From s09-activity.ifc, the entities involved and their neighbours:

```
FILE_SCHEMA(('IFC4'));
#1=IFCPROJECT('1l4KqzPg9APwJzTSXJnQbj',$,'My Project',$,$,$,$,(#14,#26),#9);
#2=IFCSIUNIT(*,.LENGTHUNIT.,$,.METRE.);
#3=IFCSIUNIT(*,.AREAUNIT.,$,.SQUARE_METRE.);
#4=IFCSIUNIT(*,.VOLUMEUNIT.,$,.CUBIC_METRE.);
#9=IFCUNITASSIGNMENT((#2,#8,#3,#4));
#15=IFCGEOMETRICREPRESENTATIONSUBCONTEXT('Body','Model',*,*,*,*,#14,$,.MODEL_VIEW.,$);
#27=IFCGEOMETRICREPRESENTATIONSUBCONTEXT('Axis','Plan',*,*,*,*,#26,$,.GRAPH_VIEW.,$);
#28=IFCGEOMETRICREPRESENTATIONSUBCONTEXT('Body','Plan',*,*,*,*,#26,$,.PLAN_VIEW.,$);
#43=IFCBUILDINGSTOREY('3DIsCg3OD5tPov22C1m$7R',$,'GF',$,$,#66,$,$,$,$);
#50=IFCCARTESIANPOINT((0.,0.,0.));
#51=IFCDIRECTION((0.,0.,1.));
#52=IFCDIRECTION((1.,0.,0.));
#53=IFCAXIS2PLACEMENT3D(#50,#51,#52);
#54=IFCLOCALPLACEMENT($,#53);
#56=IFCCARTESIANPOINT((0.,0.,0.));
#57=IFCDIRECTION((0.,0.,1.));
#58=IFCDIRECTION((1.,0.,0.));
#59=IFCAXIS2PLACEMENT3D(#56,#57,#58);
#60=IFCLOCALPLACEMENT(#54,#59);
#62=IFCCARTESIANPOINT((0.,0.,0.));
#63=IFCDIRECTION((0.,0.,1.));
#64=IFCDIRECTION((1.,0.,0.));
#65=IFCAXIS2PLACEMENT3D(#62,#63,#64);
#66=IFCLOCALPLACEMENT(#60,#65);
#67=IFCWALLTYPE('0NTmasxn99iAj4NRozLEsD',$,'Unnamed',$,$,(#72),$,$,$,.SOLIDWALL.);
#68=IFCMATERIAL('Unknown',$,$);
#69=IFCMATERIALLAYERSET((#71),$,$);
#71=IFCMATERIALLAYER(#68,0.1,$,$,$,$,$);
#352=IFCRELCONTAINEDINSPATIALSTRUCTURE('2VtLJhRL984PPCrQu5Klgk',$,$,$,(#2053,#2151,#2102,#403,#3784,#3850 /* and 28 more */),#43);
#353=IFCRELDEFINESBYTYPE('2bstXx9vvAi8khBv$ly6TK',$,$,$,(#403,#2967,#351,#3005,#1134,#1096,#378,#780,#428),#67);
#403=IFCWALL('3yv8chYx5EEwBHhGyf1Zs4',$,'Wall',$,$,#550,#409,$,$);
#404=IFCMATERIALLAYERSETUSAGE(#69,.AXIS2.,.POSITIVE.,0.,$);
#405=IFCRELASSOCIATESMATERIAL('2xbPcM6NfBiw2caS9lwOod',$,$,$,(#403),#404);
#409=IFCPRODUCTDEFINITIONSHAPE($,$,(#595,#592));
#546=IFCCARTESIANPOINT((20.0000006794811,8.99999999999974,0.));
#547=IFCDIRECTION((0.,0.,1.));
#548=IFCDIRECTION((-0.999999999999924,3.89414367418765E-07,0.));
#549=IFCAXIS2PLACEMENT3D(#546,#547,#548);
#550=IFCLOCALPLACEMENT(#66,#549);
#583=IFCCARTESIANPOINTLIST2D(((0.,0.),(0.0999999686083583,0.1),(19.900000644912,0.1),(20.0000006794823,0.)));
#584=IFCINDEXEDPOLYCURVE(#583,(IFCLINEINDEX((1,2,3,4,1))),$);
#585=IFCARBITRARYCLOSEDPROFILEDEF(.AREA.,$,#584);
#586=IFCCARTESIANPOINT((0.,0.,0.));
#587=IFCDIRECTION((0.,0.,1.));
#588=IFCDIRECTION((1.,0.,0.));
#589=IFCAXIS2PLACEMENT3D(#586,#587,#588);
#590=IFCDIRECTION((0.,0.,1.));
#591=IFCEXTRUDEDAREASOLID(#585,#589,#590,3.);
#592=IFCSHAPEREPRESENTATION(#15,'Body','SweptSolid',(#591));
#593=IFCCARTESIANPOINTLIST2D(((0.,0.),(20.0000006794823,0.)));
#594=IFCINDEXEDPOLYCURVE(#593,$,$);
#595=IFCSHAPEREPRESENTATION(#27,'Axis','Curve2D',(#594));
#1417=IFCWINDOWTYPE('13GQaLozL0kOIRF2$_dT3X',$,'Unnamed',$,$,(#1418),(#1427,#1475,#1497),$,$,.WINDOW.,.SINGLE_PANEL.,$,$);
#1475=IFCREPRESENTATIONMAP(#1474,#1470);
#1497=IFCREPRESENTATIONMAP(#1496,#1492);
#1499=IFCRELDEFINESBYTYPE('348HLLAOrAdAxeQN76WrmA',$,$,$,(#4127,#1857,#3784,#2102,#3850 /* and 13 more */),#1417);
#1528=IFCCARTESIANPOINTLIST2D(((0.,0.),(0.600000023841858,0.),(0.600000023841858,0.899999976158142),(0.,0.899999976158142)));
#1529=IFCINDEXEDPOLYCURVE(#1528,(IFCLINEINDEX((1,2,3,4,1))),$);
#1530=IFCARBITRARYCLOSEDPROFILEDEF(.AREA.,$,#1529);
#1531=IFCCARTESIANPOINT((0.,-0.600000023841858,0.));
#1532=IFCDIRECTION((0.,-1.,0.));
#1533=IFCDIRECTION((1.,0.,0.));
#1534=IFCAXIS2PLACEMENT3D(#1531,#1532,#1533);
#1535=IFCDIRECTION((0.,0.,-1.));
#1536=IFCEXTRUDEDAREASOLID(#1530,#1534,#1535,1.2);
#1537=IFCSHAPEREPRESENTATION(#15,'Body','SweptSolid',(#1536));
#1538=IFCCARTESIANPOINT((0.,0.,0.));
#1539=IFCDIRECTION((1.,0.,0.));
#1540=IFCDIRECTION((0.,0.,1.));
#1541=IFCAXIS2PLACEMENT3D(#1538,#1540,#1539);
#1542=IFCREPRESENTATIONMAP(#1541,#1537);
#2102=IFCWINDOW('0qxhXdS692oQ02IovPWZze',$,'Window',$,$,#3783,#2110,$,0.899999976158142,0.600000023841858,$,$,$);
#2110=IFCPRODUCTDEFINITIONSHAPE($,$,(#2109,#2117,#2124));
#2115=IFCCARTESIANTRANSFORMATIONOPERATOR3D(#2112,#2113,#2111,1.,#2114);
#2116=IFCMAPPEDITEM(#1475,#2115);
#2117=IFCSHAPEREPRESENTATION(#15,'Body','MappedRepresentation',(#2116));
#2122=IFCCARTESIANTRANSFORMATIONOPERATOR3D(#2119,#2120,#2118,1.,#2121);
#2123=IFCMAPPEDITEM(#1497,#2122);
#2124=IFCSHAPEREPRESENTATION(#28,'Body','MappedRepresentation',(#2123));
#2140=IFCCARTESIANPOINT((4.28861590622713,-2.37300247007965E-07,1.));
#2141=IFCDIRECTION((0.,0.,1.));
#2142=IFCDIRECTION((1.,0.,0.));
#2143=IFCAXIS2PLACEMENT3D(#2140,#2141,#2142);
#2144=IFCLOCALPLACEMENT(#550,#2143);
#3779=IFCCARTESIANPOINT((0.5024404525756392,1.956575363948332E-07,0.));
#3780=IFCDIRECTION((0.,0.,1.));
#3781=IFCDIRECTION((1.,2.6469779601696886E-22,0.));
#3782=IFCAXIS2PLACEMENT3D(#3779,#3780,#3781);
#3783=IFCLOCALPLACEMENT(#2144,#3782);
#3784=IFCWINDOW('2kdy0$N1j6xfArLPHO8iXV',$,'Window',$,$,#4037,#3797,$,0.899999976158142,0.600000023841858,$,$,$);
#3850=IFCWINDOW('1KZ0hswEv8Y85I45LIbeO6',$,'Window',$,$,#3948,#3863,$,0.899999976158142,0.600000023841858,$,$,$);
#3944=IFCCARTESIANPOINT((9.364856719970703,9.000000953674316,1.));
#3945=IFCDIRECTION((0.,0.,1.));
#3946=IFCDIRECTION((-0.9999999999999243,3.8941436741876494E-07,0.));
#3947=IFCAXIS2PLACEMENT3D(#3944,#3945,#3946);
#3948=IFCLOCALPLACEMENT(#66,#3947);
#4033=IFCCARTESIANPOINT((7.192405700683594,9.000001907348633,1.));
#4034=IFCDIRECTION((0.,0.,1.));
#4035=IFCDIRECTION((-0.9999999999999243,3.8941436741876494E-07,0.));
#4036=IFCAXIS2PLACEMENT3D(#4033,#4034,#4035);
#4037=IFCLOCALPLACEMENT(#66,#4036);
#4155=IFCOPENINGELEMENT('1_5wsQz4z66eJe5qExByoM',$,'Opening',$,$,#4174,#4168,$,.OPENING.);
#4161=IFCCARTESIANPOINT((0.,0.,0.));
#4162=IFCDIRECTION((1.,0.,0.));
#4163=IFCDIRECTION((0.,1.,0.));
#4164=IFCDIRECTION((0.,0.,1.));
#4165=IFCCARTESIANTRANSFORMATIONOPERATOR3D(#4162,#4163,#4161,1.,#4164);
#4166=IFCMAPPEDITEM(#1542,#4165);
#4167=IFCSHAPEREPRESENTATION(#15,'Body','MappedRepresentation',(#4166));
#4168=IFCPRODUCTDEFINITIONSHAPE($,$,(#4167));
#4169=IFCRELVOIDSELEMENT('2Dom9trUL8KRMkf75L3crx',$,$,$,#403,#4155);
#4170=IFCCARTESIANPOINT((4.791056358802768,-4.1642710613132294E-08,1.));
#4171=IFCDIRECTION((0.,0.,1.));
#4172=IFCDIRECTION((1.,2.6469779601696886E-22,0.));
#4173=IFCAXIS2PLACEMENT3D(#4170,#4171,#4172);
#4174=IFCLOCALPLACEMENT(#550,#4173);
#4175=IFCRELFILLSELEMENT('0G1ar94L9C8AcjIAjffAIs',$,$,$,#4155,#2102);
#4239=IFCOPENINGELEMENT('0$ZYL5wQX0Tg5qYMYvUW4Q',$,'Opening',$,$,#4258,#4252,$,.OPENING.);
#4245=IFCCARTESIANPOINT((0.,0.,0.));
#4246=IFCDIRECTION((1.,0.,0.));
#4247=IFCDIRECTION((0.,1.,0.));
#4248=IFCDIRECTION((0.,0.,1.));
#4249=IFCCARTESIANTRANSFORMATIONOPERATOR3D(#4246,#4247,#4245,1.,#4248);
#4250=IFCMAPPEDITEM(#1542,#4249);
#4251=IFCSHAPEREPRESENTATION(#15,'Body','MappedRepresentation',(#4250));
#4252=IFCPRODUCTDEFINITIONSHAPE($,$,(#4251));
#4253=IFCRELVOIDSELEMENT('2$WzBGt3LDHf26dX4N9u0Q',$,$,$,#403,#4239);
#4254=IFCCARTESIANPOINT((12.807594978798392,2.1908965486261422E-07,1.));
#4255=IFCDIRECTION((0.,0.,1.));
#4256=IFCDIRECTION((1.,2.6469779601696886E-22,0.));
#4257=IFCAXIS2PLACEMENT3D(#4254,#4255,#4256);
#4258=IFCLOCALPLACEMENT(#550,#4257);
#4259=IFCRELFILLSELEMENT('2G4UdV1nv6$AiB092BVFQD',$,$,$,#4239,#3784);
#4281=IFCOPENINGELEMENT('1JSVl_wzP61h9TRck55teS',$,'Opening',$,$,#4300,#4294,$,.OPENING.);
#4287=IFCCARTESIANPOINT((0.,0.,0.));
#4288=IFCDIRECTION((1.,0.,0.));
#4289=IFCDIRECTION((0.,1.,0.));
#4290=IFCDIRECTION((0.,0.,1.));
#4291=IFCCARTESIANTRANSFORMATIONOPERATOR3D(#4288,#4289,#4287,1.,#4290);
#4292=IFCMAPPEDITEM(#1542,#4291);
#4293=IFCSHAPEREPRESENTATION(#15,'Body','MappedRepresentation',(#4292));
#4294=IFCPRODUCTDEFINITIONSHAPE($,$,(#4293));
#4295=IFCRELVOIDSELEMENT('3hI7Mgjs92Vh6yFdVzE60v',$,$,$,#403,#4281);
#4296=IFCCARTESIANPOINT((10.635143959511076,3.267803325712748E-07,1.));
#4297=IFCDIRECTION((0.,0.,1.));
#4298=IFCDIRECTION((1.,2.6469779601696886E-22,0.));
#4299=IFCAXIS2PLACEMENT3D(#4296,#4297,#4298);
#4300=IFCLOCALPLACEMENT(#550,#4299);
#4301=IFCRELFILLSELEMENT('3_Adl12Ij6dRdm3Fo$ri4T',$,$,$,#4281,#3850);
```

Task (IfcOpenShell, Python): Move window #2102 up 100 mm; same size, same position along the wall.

```python
import numpy as np
import ifcopenshell
import ifcopenshell.api.geometry
import ifcopenshell.util.placement
import ifcopenshell.util.unit

model = ifcopenshell.open("s09-activity.ifc")
unit_scale = ifcopenshell.util.unit.calculate_unit_scale(model)

window = model.by_id(2102)
opening = window.FillsVoids[0].RelatingOpeningElement
dz = 0.1 / unit_scale

shift = np.array([0.0, 0.0, dz])
# The window is not placed relative to its opening, so move both.
for product in (opening, window):
    matrix = ifcopenshell.util.placement.get_local_placement(product.ObjectPlacement)
    matrix[:3, 3] += shift
    ifcopenshell.api.geometry.edit_object_placement(model, product=product, matrix=matrix, is_si=False)

print(f"moved by {dz * unit_scale:+.3f} m")

model.write("s09-activity-out.ifc")
```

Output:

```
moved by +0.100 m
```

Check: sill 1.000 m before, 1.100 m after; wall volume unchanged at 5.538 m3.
